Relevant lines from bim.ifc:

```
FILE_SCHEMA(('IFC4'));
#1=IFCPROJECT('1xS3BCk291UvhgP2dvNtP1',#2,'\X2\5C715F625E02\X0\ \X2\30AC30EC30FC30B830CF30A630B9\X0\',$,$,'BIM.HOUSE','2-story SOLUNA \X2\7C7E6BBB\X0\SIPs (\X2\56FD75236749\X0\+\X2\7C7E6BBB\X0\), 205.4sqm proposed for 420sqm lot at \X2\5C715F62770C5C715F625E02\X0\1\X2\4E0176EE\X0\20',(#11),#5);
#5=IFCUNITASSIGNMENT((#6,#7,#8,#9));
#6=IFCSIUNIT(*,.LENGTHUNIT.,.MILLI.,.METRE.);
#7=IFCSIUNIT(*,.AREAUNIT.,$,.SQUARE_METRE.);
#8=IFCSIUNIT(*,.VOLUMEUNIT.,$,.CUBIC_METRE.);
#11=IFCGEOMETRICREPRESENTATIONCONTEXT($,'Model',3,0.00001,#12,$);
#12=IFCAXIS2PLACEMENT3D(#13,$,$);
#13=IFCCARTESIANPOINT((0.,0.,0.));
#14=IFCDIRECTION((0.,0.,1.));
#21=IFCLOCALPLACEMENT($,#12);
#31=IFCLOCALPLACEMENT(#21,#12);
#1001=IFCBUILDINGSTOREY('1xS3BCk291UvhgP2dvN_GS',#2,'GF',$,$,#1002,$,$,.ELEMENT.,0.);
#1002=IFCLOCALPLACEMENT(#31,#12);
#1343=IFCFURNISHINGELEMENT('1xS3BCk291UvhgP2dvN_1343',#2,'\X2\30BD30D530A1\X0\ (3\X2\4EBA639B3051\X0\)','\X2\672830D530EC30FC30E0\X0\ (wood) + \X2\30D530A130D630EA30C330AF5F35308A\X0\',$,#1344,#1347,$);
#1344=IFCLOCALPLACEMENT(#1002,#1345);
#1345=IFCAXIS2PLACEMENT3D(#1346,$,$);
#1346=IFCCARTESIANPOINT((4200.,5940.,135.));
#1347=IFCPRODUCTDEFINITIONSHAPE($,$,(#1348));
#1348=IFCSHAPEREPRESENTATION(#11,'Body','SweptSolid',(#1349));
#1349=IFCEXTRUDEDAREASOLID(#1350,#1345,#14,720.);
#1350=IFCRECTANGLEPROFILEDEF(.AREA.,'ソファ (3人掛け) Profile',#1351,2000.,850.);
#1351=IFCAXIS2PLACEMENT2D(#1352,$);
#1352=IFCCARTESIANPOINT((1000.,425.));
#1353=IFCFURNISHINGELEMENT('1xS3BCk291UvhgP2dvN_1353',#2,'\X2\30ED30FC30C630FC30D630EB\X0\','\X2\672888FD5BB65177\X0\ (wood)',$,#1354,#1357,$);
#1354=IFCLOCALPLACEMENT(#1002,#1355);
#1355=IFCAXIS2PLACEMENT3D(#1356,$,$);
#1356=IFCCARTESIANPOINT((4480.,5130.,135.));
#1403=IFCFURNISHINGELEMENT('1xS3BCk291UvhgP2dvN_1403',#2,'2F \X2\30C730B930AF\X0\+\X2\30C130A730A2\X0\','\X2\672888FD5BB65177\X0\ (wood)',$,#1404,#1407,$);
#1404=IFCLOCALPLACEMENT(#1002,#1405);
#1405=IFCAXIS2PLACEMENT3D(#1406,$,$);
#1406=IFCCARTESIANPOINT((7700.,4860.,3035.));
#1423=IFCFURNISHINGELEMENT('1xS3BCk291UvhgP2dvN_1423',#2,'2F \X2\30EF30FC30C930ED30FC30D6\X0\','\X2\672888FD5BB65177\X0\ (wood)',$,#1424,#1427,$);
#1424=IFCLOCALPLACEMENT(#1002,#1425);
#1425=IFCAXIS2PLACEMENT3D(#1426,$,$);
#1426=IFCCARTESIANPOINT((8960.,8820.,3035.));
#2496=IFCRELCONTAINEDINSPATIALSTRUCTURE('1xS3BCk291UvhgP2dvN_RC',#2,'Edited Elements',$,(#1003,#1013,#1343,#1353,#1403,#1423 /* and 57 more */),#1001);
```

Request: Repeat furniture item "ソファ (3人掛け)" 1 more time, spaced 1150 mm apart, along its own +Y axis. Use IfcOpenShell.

```python
import ifcopenshell
import ifcopenshell.api.geometry
import ifcopenshell.api.root
import ifcopenshell.util.element
import ifcopenshell.util.placement
import ifcopenshell.util.unit

model = ifcopenshell.open("bim.ifc")
unit_scale = ifcopenshell.util.unit.calculate_unit_scale(model)


def reuse_history(source, copy):
    """copy_class also copies each property set's owner history, people and application; keep the originals."""
    for rel in copy.IsDefinedBy:
        if rel.is_a("IfcRelDefinesByProperties") and (history := rel.RelatingPropertyDefinition.OwnerHistory):
            rel.RelatingPropertyDefinition.OwnerHistory = source.OwnerHistory
            ifcopenshell.util.element.remove_deep2(model, history)


source = model.by_guid("1xS3BCk291UvhgP2dvN_1343")
base = ifcopenshell.util.placement.get_local_placement(source.ObjectPlacement)
step = base[:3, 1] * 1.15 / unit_scale

for i in range(1, 2):
    copy = ifcopenshell.api.root.copy_class(model, product=source)
    copy.Representation = ifcopenshell.util.element.copy_deep(
        model, source.Representation, exclude=["IfcGeometricRepresentationContext", "IfcRepresentationMap"]
    )
    reuse_history(source, copy)
    matrix = base.copy()
    matrix[:3, 3] += i * step
    print("added at", matrix[:3, 3].round(3) + 0.0)
    ifcopenshell.api.geometry.edit_object_placement(model, product=copy, matrix=matrix, is_si=False)

model.write("bim_v2.ifc")
```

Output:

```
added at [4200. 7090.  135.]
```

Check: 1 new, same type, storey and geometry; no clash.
